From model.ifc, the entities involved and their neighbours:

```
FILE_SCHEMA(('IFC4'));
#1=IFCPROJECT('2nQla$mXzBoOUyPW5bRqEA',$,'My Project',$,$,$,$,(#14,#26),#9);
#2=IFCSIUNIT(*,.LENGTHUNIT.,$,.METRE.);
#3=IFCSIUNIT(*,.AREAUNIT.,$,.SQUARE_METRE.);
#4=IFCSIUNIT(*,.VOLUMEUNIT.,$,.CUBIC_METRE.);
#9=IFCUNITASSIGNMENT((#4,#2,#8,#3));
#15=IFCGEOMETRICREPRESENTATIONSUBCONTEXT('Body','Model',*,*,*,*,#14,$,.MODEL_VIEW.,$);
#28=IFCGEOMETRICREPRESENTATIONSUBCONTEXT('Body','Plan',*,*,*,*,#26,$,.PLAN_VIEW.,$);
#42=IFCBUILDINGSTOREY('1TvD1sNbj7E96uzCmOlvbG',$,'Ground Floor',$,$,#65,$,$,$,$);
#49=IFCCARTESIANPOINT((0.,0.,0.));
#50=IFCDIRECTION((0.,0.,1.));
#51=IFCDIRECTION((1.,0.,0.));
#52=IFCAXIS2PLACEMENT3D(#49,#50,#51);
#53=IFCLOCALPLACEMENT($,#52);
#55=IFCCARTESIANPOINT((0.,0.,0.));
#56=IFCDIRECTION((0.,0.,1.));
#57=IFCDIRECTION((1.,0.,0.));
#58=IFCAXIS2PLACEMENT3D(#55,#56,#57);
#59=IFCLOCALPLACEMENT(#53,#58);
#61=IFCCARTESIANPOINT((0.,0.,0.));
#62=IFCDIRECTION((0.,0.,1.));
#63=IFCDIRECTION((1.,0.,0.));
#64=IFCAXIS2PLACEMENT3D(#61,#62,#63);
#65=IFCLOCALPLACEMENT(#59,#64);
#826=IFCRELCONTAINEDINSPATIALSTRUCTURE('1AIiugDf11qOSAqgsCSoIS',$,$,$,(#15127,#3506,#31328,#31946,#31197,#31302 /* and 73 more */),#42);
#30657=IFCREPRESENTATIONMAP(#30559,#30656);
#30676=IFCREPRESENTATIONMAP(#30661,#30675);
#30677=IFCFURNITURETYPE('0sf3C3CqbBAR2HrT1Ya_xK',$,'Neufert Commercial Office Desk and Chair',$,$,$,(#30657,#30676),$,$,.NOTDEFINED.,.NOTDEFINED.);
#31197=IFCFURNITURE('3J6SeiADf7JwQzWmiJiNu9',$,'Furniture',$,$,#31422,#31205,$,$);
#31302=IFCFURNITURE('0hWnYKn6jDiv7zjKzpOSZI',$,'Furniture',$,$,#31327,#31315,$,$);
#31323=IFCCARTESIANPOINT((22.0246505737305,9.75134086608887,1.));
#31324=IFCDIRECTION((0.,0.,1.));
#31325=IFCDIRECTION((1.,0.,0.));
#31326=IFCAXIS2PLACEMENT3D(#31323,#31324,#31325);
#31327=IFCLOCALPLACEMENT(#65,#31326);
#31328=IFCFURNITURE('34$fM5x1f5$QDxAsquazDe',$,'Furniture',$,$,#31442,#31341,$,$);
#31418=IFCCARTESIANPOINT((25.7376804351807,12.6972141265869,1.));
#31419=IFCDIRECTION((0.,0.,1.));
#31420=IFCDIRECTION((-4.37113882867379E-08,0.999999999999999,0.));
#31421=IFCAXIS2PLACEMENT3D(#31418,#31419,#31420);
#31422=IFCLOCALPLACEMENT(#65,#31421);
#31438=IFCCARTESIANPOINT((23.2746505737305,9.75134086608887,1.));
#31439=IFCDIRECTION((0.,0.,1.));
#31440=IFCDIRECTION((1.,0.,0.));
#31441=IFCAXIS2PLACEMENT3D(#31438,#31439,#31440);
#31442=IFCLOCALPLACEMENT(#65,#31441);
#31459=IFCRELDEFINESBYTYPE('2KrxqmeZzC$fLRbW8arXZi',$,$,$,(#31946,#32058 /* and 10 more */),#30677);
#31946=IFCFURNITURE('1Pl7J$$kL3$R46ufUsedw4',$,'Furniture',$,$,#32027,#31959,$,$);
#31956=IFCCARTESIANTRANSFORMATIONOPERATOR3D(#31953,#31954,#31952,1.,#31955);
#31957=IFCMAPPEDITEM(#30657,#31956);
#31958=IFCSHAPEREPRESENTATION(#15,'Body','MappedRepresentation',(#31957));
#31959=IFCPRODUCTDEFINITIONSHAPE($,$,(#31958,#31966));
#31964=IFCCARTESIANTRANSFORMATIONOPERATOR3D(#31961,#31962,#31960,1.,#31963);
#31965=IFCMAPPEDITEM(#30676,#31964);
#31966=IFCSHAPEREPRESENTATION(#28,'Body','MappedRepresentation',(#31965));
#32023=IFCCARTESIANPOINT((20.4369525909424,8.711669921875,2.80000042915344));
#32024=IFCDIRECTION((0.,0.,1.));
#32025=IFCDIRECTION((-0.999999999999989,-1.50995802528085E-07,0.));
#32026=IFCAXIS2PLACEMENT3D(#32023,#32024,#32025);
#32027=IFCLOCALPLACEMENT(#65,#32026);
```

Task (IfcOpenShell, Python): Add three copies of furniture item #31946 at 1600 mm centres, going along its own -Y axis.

```python
import ifcopenshell
import ifcopenshell.api.geometry
import ifcopenshell.api.root
import ifcopenshell.util.element
import ifcopenshell.util.placement
import ifcopenshell.util.unit

model = ifcopenshell.open("model.ifc")
unit_scale = ifcopenshell.util.unit.calculate_unit_scale(model)

source = model.by_guid("1Pl7J$$kL3$R46ufUsedw4")
base = ifcopenshell.util.placement.get_local_placement(source.ObjectPlacement)
step = -base[:3, 1] * 1.6 / unit_scale

for i in range(1, 4):
    copy = ifcopenshell.api.root.copy_class(model, product=source)
    copy.Representation = ifcopenshell.util.element.copy_deep(
        model, source.Representation, exclude=["IfcGeometricRepresentationContext", "IfcRepresentationMap"]
    )
    matrix = base.copy()
    matrix[:3, 3] += i * step
    print("added at", matrix[:3, 3].round(3) + 0.0)
    ifcopenshell.api.geometry.edit_object_placement(model, product=copy, matrix=matrix, is_si=False)

model.write("model_v2.ifc")
```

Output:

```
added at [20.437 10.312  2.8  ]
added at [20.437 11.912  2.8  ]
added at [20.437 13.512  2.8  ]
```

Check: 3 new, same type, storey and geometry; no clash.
